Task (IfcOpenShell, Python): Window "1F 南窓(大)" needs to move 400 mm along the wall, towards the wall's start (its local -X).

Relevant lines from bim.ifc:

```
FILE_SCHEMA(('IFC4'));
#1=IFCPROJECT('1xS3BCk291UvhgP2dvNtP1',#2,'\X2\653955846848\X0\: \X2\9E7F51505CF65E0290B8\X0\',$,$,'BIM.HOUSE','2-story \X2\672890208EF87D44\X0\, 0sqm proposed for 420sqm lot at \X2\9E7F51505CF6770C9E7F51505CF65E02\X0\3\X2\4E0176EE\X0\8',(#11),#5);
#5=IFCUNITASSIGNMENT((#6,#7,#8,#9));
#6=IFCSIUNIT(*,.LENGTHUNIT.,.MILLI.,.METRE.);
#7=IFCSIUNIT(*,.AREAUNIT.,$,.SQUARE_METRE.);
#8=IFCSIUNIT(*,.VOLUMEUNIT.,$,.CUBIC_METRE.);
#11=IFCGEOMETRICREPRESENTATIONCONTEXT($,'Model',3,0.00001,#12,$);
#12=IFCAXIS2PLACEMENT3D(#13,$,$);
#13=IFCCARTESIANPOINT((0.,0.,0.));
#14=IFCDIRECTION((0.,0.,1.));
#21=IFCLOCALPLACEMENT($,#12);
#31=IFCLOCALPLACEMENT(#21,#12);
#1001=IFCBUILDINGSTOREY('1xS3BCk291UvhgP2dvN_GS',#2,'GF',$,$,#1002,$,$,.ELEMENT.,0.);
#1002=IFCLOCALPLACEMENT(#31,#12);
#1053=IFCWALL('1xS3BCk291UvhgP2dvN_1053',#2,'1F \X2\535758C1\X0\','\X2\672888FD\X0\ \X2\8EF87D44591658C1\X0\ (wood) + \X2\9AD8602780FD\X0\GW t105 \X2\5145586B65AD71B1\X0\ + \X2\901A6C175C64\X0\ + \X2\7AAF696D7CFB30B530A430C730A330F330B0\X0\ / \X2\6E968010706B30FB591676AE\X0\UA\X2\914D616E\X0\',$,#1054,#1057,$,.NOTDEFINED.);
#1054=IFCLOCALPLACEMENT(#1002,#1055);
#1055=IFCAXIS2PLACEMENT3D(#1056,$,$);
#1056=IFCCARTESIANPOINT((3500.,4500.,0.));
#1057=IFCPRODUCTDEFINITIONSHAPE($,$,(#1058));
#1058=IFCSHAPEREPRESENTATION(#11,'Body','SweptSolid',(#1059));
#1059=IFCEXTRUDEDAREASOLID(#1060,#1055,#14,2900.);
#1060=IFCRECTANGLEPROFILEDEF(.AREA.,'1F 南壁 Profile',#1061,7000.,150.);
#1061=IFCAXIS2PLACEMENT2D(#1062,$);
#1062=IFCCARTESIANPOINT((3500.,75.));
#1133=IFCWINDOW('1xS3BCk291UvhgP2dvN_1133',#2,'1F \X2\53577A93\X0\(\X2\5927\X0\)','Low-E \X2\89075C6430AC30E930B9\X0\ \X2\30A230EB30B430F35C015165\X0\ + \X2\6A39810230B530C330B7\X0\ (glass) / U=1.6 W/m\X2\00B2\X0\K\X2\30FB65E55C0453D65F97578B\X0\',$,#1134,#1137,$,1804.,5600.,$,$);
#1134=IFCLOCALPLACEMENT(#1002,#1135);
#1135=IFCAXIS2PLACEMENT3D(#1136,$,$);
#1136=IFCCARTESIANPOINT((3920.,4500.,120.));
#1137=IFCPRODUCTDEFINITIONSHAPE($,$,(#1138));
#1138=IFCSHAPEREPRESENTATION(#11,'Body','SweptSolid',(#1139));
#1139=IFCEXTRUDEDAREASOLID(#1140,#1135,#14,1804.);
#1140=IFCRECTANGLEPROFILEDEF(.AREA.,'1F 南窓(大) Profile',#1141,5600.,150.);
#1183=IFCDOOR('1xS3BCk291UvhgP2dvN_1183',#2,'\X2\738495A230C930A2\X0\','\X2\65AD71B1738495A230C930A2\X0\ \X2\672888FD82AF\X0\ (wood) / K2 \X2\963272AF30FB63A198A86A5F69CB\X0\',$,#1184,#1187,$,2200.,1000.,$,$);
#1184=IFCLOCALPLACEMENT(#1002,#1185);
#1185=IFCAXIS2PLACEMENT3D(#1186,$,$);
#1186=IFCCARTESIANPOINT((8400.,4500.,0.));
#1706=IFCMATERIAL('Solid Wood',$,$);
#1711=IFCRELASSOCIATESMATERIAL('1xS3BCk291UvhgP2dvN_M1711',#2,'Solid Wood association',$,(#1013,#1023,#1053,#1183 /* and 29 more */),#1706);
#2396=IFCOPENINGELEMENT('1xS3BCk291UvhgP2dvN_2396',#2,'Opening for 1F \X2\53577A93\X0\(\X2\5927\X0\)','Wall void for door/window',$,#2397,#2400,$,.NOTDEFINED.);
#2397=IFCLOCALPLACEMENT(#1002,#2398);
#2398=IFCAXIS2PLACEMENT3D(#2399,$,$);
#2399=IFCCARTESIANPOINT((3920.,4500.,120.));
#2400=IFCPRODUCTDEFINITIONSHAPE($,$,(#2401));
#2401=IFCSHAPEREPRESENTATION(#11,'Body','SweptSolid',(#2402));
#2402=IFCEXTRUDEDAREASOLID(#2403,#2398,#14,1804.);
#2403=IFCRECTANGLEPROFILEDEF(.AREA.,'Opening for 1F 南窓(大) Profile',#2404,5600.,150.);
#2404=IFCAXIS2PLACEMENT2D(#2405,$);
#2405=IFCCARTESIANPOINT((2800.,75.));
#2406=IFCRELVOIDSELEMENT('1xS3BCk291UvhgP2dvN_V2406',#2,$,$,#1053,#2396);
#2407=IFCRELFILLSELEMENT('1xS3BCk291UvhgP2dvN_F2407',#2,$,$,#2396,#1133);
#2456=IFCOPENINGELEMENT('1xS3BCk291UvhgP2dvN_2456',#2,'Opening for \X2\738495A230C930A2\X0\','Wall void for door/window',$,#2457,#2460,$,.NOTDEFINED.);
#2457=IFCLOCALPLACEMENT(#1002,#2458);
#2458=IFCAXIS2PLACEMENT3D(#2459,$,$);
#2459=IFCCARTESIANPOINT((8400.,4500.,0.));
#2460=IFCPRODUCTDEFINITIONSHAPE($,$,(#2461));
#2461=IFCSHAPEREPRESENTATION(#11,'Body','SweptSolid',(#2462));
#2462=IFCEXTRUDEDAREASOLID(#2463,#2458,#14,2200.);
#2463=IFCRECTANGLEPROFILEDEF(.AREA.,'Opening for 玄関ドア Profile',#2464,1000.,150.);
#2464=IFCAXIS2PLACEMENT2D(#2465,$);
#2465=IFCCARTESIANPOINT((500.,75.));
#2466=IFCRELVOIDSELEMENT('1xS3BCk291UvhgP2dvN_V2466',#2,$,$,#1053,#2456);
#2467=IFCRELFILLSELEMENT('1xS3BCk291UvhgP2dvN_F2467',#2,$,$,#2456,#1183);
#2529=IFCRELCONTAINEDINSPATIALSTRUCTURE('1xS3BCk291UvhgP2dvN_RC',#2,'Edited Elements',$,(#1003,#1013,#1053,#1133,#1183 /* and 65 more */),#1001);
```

```python
import ifcopenshell
import ifcopenshell.api.geometry
import ifcopenshell.util.placement
import ifcopenshell.util.unit

model = ifcopenshell.open("bim.ifc")
unit_scale = ifcopenshell.util.unit.calculate_unit_scale(model)

window = model.by_guid("1xS3BCk291UvhgP2dvN_1133")
opening = window.FillsVoids[0].RelatingOpeningElement
wall = opening.VoidsElements[0].RelatingBuildingElement

wall_matrix = ifcopenshell.util.placement.get_local_placement(wall.ObjectPlacement)
shift = wall_matrix[:3, 0] * -0.4 / unit_scale
before = ifcopenshell.util.placement.get_local_placement(window.ObjectPlacement)[:3, 3].copy()

# The window is not placed relative to its opening, so move both.
for product in (opening, window):
    matrix = ifcopenshell.util.placement.get_local_placement(product.ObjectPlacement)
    matrix[:3, 3] += shift
    ifcopenshell.api.geometry.edit_object_placement(model, product=product, matrix=matrix, is_si=False)

after = ifcopenshell.util.placement.get_local_placement(window.ObjectPlacement)[:3, 3]
print("window moved by", (after - before).round(3) + 0.0)

model.write("bim_edited.ifc")
```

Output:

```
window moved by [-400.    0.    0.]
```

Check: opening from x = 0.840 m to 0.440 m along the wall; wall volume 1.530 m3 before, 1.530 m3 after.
